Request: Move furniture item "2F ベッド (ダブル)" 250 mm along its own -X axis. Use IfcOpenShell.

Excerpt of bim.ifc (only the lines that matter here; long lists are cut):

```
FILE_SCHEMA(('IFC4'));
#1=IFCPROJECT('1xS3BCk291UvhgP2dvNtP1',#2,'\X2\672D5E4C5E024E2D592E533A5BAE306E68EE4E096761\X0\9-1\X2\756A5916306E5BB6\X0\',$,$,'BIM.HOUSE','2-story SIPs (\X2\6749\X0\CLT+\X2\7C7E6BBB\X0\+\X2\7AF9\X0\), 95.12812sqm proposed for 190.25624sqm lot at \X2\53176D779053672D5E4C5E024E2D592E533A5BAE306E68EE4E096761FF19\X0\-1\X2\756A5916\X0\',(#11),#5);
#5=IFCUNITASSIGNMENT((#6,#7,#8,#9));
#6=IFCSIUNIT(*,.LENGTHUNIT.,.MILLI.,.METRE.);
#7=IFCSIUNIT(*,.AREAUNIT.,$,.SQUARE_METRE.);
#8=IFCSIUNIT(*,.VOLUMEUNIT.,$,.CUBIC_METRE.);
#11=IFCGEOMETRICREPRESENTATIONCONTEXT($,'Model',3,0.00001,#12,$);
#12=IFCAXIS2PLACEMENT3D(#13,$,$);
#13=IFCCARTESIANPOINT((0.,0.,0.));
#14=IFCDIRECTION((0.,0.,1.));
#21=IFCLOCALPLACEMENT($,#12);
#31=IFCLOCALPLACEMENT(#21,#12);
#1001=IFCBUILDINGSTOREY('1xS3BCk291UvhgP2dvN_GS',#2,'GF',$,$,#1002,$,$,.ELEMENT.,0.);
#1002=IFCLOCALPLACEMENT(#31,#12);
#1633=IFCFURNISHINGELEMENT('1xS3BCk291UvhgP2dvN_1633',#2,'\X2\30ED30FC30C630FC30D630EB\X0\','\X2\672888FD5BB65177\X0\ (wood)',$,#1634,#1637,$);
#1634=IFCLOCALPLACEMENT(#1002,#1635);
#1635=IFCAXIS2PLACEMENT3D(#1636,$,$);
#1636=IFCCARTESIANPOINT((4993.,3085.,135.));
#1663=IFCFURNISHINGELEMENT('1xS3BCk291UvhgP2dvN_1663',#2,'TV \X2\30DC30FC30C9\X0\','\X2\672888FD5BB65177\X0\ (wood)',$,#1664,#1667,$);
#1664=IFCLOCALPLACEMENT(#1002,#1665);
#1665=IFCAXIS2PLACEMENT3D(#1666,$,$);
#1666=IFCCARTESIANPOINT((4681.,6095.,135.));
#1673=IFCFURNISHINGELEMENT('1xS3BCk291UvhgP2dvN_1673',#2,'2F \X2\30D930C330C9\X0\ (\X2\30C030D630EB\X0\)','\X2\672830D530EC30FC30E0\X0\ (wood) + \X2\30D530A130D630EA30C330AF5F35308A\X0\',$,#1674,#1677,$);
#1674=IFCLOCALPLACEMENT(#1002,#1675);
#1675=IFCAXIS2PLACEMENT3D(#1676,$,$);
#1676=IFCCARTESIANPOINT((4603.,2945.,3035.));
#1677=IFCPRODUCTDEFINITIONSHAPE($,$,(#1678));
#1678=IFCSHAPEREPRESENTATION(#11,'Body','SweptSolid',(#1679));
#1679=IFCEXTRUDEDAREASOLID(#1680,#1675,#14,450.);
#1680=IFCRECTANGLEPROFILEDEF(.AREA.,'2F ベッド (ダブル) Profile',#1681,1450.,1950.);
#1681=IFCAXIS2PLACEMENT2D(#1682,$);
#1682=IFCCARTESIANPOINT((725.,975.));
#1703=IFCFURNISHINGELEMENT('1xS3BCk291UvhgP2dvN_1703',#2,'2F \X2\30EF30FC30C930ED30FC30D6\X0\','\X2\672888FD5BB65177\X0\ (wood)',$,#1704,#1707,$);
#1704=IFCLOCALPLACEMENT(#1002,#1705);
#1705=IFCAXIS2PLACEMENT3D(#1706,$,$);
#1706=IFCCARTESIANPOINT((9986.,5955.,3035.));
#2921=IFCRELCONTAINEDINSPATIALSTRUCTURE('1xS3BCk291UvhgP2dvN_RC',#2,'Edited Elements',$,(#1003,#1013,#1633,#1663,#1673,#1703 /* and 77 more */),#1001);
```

```python
import ifcopenshell
import ifcopenshell.api.geometry
import ifcopenshell.util.placement

model = ifcopenshell.open("bim.ifc")

item = model.by_id(1673)
matrix = ifcopenshell.util.placement.get_local_placement(item.ObjectPlacement)
matrix[:3, 3] -= matrix[:3, 0] * 250.0
ifcopenshell.api.geometry.edit_object_placement(model, product=item, matrix=matrix, is_si=False)

print(ifcopenshell.util.placement.get_local_placement(item.ObjectPlacement).round(3) + 0.0)

model.write("bim_v2.ifc")
```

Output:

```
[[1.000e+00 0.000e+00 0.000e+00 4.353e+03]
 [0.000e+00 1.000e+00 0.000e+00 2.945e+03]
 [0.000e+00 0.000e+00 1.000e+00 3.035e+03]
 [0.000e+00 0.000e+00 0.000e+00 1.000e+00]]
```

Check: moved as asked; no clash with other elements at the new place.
